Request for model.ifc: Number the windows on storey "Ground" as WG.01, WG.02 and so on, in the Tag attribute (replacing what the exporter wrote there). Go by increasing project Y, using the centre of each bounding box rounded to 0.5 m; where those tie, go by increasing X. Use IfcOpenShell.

First a look at what the model holds.

```python
import ifcopenshell
import ifcopenshell.util.element
import ifcopenshell.util.placement

model = ifcopenshell.open("model.ifc")
print(model.schema)
storey = next(s for s in model.by_type("IfcBuildingStorey") if s.Name == "Ground")
windows = [e for e in ifcopenshell.util.element.get_decomposition(storey) if e.is_a("IfcWindow")]
for e in sorted(windows, key=lambda e: e.id()):
    origin = ifcopenshell.util.placement.get_local_placement(e.ObjectPlacement)[:3, 3]
    print(e.id(), e.Tag, e.Name, origin.round(2) + 0.0, sep=" | ")
```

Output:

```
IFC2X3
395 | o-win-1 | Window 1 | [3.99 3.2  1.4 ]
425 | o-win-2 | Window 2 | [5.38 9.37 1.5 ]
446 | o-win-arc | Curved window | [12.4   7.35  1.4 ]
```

```python
import ifcopenshell
import ifcopenshell.geom
import ifcopenshell.util.element
import ifcopenshell.util.shape

model = ifcopenshell.open("model.ifc")
settings = ifcopenshell.geom.settings()
settings.set("use-world-coords", True)


def centre(element):
    shape = ifcopenshell.geom.create_shape(settings, element)
    return ifcopenshell.util.shape.get_bbox_centroid(shape.geometry)


storey = next(s for s in model.by_type("IfcBuildingStorey") if s.Name == "Ground")
windows = [e for e in ifcopenshell.util.element.get_decomposition(storey) if e.is_a("IfcWindow")]

# Insertion points can sit at a corner or the storey origin, so sort by the geometry (in metres).
centres = {e: centre(e) for e in windows}
windows.sort(key=lambda e: (round(centres[e][1] / 0.5), centres[e][0]))

for i, e in enumerate(windows, start=1):
    number = f"WG.{i:02d}"
    e.Tag = number
    print(e.id(), number)

model.write("model_edited.ifc")
```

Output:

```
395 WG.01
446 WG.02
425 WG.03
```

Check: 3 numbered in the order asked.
